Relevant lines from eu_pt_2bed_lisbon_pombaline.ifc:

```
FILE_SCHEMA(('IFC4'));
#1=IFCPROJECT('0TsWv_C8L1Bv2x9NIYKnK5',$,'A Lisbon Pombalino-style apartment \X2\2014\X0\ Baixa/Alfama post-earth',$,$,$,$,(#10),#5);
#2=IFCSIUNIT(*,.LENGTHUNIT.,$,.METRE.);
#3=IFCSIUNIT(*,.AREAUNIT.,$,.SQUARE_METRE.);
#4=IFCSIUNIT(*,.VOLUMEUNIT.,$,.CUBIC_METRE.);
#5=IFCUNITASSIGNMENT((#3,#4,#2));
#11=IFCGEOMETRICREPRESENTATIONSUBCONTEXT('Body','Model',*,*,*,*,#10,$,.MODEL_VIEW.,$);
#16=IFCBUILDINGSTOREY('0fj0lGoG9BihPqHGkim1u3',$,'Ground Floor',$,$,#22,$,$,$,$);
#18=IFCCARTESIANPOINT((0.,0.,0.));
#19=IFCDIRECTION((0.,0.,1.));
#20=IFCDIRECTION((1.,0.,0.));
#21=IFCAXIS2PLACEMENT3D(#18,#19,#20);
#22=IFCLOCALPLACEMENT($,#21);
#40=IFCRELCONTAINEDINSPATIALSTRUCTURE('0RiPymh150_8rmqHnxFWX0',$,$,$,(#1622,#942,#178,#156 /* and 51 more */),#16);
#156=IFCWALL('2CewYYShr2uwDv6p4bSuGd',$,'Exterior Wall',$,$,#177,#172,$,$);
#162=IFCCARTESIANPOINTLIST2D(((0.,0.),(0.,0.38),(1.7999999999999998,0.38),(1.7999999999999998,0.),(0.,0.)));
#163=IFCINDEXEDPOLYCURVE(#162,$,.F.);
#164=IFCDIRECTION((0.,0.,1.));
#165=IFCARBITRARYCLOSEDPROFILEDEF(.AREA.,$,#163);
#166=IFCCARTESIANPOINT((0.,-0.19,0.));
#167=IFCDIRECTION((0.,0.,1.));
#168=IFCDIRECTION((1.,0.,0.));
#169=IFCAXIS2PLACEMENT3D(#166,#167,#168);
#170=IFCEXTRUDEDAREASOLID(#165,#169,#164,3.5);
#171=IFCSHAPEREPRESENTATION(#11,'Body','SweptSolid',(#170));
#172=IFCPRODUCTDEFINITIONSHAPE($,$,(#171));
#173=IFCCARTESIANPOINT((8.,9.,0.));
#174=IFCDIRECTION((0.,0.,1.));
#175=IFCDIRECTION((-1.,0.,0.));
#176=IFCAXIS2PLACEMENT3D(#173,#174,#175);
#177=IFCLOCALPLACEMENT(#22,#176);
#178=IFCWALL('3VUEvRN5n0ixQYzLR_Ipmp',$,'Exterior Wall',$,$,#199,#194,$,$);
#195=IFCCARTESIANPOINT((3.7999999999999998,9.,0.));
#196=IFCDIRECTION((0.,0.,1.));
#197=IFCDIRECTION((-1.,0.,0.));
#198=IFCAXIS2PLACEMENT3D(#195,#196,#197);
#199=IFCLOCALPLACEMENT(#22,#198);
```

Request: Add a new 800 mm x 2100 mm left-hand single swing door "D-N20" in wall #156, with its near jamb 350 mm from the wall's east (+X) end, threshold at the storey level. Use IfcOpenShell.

```python
import numpy as np
import ifcopenshell
import ifcopenshell.api.feature
import ifcopenshell.api.geometry
import ifcopenshell.api.root
import ifcopenshell.api.spatial
import ifcopenshell.geom
import ifcopenshell.util.element
import ifcopenshell.util.placement
import ifcopenshell.util.representation
import ifcopenshell.util.shape
import ifcopenshell.util.unit

model = ifcopenshell.open("eu_pt_2bed_lisbon_pombaline.ifc")
unit_scale = ifcopenshell.util.unit.calculate_unit_scale(model)
settings = ifcopenshell.geom.settings()


def volume(element):
    """Net volume in cubic metres, openings subtracted."""
    shape = ifcopenshell.geom.create_shape(settings, element)
    return ifcopenshell.util.shape.get_volume(shape.geometry)


wall = model.by_guid("2CewYYShr2uwDv6p4bSuGd")
storey = ifcopenshell.util.element.get_container(wall, ifc_class="IfcBuildingStorey")
context = ifcopenshell.util.representation.get_context(model, "Model", "Body", "MODEL_VIEW")
before = volume(wall)

width, height, from_end, sill = 0.8, 2.1, 0.35, 0.0  # metres

# The wall runs along its own X axis, and the end named is its -X end.
wall_shape = ifcopenshell.geom.create_shape(settings, wall)
x, y, z = ifcopenshell.util.shape.get_vertices(wall_shape.geometry).T
start = x.min() + from_end
face, thickness = float(y.min()), float(y.max() - y.min())
wall_matrix = ifcopenshell.util.placement.get_local_placement(wall.ObjectPlacement)
level = ifcopenshell.util.placement.get_local_placement(storey.ObjectPlacement)[2, 3]


def in_wall(x, y):
    """Placement at x, y metres in the wall's axes, at sill height."""
    matrix = wall_matrix.copy()
    matrix[:, 3] = wall_matrix @ np.array([x / unit_scale, y / unit_scale, 0.0, 1.0])
    matrix[2, 3] = level + sill / unit_scale
    return matrix


# Opening: a box that overshoots both wall faces by 50 mm.
opening = ifcopenshell.api.root.create_entity(model, ifc_class="IfcOpeningElement", predefined_type="OPENING")
box = ifcopenshell.api.geometry.add_wall_representation(
    model, context=context, length=width, height=height, thickness=thickness + 0.1
)
ifcopenshell.api.geometry.assign_representation(model, product=opening, representation=box)
ifcopenshell.api.geometry.edit_object_placement(model, product=opening, matrix=in_wall(start, face - 0.05), is_si=False)
ifcopenshell.api.feature.add_feature(model, feature=opening, element=wall)

door = ifcopenshell.api.root.create_entity(model, ifc_class="IfcDoor", name="D-N20", predefined_type="DOOR")
door.OverallWidth, door.OverallHeight = width / unit_scale, height / unit_scale
door.OperationType = "SINGLE_SWING_LEFT"
body = ifcopenshell.api.geometry.add_door_representation(
    model,
    context=context,
    overall_width=door.OverallWidth,
    overall_height=door.OverallHeight,
    operation_type="SINGLE_SWING_LEFT",
    lining_properties={"LiningDepth": thickness / unit_scale, "ThresholdDepth": thickness / unit_scale},
)
ifcopenshell.api.geometry.assign_representation(model, product=door, representation=body)
ifcopenshell.api.spatial.assign_container(model, products=[door], relating_structure=storey)
ifcopenshell.api.feature.add_filling(model, opening=opening, element=door)

# The lining spans the wall, so the door starts at the wall face.
ifcopenshell.api.geometry.edit_object_placement(model, product=door, matrix=in_wall(start, face), is_si=False)

after = volume(wall)

print(f"wall volume {before:.3f} -> {after:.3f} m3")

model.write("eu_pt_2bed_lisbon_pombaline_v2.ifc")
```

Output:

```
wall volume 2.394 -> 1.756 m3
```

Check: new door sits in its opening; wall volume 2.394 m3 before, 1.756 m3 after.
